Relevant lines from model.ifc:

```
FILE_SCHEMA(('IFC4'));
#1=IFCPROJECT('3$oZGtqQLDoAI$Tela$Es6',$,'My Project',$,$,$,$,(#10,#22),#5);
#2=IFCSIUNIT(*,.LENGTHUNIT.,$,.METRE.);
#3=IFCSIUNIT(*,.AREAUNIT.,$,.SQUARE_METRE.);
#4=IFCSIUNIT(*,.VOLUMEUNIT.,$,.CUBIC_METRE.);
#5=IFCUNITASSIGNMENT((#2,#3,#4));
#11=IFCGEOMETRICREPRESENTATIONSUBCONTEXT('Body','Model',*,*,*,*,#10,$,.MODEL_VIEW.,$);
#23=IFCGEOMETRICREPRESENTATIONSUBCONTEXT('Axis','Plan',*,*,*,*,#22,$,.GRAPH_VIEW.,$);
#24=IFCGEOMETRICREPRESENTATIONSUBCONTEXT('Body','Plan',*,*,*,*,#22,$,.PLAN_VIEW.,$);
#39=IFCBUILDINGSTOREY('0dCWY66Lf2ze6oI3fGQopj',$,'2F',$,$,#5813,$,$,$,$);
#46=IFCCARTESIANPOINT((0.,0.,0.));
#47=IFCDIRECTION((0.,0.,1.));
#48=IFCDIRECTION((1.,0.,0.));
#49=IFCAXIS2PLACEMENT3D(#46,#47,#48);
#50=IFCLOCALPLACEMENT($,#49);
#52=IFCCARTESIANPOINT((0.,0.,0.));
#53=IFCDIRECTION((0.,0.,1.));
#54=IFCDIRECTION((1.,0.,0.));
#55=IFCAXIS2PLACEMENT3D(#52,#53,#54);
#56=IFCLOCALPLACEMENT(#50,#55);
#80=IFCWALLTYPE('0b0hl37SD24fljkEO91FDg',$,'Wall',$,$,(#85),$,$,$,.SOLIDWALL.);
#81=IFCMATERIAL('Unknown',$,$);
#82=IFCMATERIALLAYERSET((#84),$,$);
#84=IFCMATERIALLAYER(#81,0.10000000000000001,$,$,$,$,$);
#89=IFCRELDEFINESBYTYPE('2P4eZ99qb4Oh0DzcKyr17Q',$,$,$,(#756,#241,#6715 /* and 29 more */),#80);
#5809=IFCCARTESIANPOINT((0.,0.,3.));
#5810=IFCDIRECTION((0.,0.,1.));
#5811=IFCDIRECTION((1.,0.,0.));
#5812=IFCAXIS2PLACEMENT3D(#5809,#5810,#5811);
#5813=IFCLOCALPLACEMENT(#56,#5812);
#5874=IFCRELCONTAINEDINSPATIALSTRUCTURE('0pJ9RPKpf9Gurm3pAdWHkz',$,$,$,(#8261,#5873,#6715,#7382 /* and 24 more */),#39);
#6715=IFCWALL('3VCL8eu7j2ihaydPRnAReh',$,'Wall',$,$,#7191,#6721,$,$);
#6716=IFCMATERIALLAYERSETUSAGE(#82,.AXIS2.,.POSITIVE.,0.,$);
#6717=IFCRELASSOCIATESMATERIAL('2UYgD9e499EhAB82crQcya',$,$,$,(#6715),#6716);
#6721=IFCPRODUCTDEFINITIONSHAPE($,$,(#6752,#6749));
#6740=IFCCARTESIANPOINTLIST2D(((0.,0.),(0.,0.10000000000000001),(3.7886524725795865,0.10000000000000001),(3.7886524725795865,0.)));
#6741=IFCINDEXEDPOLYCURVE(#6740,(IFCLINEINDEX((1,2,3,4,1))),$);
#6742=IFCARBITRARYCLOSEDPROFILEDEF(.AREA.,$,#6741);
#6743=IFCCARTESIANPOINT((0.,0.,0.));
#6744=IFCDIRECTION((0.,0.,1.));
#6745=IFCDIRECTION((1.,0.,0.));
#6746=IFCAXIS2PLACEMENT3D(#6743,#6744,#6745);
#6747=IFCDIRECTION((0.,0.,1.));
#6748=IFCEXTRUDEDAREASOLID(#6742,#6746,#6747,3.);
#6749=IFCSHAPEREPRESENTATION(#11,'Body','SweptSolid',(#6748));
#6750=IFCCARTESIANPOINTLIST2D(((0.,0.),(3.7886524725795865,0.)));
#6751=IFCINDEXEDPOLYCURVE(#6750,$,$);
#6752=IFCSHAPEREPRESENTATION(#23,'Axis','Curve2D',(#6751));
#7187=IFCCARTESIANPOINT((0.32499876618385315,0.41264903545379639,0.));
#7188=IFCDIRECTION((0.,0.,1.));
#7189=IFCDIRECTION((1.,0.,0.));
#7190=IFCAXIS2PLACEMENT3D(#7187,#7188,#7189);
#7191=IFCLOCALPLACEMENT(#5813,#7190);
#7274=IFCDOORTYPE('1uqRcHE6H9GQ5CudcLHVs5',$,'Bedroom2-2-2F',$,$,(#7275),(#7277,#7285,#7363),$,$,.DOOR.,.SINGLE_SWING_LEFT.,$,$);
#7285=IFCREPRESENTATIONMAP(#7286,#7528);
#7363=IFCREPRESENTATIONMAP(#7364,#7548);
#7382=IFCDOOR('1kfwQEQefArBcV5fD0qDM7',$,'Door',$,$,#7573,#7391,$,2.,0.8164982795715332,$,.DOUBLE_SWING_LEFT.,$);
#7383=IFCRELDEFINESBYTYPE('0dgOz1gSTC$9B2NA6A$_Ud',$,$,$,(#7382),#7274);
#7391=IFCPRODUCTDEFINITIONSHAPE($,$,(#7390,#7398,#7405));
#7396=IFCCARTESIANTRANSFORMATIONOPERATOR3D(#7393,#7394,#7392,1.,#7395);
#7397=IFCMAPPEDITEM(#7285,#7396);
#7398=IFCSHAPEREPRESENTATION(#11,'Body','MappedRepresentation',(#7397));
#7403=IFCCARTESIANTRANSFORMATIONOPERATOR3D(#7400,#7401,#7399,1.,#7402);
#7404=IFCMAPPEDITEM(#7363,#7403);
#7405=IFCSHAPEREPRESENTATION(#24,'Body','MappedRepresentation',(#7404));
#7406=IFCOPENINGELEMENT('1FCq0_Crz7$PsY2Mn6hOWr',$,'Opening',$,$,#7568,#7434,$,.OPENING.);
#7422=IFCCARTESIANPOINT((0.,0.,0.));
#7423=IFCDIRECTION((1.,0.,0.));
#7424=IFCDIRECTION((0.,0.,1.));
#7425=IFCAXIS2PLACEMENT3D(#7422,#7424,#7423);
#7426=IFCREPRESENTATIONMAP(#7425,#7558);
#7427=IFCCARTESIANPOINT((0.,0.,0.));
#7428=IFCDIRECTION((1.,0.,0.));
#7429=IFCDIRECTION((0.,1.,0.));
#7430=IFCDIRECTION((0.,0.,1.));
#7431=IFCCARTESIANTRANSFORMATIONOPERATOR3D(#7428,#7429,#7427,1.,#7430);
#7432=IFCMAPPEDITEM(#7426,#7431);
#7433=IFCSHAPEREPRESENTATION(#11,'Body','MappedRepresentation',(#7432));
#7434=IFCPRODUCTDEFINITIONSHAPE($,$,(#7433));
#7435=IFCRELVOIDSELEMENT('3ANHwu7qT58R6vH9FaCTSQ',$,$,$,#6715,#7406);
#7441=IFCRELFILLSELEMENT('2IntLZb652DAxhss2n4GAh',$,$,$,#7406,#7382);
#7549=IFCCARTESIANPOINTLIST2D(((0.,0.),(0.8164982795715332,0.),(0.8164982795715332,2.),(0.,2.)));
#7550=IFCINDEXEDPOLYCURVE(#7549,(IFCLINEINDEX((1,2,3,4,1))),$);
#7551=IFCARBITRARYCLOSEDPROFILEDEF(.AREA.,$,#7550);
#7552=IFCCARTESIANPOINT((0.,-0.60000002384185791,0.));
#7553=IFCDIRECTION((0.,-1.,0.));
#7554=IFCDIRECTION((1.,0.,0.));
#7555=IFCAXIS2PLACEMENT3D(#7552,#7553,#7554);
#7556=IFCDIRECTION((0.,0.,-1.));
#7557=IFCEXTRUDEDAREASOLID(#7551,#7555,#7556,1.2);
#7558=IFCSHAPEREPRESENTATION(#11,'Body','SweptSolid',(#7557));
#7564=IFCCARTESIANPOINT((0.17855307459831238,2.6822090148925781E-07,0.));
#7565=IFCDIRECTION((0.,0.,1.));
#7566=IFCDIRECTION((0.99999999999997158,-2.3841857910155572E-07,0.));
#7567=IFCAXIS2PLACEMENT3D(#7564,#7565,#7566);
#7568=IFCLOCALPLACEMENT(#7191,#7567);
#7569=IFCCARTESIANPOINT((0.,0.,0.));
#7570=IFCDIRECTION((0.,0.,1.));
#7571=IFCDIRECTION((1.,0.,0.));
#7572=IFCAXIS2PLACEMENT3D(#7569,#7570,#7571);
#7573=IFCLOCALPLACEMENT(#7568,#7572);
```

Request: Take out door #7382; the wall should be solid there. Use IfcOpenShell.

```python
import ifcopenshell
import ifcopenshell.api.feature
import ifcopenshell.api.root
import ifcopenshell.geom
import ifcopenshell.util.shape

model = ifcopenshell.open("model.ifc")
settings = ifcopenshell.geom.settings()


def volume(element):
    """Net volume in cubic metres, openings subtracted."""
    shape = ifcopenshell.geom.create_shape(settings, element)
    return ifcopenshell.util.shape.get_volume(shape.geometry)


door = model.by_guid("1kfwQEQefArBcV5fD0qDM7")
opening = door.FillsVoids[0].RelatingOpeningElement
wall = opening.VoidsElements[0].RelatingBuildingElement
before = volume(wall)

ifcopenshell.api.root.remove_product(model, product=door)
ifcopenshell.api.feature.remove_feature(model, feature=opening)

after = volume(wall)

print(f"wall volume {before:.3f} -> {after:.3f} m3")

model.write("model_v2.ifc")
```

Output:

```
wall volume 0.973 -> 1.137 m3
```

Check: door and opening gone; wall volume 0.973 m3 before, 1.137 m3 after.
